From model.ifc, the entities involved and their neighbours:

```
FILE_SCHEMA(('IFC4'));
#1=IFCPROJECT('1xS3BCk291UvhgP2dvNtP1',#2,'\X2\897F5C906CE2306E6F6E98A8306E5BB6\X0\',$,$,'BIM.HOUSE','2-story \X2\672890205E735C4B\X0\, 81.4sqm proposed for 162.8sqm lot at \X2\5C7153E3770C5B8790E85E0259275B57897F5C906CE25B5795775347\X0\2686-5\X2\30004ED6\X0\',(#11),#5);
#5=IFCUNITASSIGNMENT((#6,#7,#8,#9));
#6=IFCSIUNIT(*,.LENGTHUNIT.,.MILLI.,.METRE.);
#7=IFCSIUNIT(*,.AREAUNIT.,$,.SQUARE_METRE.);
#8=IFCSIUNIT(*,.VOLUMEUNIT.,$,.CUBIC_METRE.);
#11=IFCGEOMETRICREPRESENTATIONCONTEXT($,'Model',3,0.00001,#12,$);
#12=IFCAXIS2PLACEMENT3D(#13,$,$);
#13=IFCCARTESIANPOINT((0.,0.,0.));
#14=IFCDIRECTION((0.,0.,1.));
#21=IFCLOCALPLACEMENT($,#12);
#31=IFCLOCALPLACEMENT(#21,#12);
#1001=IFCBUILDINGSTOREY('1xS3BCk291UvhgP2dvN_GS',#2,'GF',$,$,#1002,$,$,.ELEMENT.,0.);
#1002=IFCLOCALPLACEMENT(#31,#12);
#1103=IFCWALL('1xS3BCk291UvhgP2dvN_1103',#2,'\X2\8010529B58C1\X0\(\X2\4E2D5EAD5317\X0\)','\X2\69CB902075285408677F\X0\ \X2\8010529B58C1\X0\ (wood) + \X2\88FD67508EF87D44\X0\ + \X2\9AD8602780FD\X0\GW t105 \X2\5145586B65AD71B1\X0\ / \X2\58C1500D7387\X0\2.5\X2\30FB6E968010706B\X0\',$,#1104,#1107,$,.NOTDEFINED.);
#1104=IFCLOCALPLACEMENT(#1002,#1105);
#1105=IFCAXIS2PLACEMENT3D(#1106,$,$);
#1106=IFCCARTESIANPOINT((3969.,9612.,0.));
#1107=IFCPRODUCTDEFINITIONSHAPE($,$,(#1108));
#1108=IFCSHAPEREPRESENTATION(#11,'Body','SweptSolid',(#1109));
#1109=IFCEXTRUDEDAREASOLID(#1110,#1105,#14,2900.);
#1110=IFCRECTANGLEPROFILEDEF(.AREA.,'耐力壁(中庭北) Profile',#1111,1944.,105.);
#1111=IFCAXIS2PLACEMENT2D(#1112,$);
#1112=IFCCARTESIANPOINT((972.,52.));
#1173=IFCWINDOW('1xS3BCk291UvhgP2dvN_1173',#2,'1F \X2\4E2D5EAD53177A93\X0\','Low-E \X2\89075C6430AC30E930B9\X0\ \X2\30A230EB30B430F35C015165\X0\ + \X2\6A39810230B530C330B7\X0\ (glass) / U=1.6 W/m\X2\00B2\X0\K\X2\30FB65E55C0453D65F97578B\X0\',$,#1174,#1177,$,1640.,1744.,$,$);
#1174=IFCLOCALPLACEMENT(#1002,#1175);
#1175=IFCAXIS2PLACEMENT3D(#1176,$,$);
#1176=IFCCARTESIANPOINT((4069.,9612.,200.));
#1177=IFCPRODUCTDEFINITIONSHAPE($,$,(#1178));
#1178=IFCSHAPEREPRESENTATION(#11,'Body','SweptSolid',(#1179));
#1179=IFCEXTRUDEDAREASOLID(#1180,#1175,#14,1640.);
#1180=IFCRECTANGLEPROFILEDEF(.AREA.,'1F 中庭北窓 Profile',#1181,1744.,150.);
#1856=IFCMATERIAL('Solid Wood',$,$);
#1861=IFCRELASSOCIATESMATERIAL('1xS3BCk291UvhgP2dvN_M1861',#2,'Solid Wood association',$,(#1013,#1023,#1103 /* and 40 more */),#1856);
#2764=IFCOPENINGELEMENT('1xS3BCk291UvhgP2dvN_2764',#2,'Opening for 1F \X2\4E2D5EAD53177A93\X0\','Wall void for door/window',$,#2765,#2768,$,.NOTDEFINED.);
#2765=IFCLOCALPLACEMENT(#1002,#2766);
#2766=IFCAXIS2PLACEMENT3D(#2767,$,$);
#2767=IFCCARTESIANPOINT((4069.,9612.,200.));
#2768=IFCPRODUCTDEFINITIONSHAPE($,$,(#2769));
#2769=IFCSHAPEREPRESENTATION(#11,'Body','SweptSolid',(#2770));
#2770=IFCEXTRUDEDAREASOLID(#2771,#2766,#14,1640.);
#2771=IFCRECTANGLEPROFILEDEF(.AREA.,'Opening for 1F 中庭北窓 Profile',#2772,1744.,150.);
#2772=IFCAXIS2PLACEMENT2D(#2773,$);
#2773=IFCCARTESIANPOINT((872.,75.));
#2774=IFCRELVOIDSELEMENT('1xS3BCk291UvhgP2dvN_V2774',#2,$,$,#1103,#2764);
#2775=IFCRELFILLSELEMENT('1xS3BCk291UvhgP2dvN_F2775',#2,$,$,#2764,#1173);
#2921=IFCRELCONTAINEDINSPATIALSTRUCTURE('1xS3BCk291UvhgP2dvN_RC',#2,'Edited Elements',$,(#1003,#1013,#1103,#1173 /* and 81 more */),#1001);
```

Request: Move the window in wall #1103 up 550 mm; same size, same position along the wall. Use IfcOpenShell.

```python
import numpy as np
import ifcopenshell
import ifcopenshell.api.geometry
import ifcopenshell.util.placement
import ifcopenshell.util.unit

model = ifcopenshell.open("model.ifc")
unit_scale = ifcopenshell.util.unit.calculate_unit_scale(model)

window = model.by_id(1173)
opening = window.FillsVoids[0].RelatingOpeningElement
dz = 0.55 / unit_scale

shift = np.array([0.0, 0.0, dz])
# The window is not placed relative to its opening, so move both.
for product in (opening, window):
    matrix = ifcopenshell.util.placement.get_local_placement(product.ObjectPlacement)
    matrix[:3, 3] += shift
    ifcopenshell.api.geometry.edit_object_placement(model, product=product, matrix=matrix, is_si=False)

print(f"moved by {dz * unit_scale:+.3f} m")

model.write("model_edited.ifc")
```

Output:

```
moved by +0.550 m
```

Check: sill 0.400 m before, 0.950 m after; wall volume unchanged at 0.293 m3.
